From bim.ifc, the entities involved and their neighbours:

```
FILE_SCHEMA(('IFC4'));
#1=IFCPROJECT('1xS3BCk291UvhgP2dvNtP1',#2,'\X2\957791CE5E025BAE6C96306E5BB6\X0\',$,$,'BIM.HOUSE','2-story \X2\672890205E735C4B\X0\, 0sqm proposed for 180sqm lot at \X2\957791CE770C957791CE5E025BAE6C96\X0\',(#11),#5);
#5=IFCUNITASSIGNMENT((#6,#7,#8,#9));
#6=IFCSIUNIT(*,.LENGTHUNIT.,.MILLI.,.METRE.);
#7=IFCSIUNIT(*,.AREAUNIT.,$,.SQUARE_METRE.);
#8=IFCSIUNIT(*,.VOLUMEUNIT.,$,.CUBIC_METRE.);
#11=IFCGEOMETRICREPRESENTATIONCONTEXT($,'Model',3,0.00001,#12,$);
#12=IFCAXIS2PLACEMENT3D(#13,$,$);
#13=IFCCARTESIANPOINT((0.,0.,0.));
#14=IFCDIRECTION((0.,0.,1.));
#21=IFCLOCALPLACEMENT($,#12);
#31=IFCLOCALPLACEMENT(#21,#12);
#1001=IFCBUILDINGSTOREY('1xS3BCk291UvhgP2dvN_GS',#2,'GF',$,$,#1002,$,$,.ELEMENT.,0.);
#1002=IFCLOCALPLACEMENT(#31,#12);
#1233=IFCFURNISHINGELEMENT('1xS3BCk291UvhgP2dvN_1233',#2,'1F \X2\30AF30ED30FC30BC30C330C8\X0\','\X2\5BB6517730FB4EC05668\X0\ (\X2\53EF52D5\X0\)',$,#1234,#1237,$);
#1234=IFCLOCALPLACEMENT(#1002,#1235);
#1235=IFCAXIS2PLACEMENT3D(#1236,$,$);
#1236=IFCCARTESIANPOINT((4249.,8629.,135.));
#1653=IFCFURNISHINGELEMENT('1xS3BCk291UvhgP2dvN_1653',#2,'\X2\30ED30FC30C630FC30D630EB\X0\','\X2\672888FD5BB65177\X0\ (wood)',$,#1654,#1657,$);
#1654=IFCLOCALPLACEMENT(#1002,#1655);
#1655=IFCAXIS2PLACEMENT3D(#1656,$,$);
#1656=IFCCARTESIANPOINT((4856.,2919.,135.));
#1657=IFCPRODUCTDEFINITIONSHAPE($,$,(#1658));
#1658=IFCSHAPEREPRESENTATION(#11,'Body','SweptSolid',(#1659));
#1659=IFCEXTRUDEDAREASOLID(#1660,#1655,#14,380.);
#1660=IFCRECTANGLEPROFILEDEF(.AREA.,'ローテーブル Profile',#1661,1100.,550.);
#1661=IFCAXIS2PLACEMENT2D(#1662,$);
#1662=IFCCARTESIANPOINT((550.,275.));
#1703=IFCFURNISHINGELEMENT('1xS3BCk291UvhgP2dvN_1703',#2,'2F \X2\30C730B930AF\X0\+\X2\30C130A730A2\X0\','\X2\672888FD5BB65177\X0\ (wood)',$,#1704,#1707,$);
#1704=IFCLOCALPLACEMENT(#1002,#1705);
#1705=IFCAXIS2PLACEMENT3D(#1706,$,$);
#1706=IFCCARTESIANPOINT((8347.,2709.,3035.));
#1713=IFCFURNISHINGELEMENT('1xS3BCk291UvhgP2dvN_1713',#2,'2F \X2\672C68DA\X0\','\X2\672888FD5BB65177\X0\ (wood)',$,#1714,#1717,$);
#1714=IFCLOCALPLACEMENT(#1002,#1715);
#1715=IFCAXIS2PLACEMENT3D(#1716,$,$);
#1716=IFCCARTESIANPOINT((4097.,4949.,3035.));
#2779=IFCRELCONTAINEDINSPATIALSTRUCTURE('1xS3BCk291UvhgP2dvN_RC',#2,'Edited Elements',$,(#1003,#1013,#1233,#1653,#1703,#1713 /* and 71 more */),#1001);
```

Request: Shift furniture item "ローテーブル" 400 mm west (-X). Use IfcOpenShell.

```python
import ifcopenshell
import ifcopenshell.api.geometry
import ifcopenshell.util.placement
import ifcopenshell.util.unit

model = ifcopenshell.open("bim.ifc")
unit_scale = ifcopenshell.util.unit.calculate_unit_scale(model)

item = model.by_guid("1xS3BCk291UvhgP2dvN_1653")
matrix = ifcopenshell.util.placement.get_local_placement(item.ObjectPlacement)
matrix[0, 3] -= 0.4 / unit_scale
ifcopenshell.api.geometry.edit_object_placement(model, product=item, matrix=matrix, is_si=False)

print(ifcopenshell.util.placement.get_local_placement(item.ObjectPlacement).round(3) + 0.0)

model.write("bim-out.ifc")
```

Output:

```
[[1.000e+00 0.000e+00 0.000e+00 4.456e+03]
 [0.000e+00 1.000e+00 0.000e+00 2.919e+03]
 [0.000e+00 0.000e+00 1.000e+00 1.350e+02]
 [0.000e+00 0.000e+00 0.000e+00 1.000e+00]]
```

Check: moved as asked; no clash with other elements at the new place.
